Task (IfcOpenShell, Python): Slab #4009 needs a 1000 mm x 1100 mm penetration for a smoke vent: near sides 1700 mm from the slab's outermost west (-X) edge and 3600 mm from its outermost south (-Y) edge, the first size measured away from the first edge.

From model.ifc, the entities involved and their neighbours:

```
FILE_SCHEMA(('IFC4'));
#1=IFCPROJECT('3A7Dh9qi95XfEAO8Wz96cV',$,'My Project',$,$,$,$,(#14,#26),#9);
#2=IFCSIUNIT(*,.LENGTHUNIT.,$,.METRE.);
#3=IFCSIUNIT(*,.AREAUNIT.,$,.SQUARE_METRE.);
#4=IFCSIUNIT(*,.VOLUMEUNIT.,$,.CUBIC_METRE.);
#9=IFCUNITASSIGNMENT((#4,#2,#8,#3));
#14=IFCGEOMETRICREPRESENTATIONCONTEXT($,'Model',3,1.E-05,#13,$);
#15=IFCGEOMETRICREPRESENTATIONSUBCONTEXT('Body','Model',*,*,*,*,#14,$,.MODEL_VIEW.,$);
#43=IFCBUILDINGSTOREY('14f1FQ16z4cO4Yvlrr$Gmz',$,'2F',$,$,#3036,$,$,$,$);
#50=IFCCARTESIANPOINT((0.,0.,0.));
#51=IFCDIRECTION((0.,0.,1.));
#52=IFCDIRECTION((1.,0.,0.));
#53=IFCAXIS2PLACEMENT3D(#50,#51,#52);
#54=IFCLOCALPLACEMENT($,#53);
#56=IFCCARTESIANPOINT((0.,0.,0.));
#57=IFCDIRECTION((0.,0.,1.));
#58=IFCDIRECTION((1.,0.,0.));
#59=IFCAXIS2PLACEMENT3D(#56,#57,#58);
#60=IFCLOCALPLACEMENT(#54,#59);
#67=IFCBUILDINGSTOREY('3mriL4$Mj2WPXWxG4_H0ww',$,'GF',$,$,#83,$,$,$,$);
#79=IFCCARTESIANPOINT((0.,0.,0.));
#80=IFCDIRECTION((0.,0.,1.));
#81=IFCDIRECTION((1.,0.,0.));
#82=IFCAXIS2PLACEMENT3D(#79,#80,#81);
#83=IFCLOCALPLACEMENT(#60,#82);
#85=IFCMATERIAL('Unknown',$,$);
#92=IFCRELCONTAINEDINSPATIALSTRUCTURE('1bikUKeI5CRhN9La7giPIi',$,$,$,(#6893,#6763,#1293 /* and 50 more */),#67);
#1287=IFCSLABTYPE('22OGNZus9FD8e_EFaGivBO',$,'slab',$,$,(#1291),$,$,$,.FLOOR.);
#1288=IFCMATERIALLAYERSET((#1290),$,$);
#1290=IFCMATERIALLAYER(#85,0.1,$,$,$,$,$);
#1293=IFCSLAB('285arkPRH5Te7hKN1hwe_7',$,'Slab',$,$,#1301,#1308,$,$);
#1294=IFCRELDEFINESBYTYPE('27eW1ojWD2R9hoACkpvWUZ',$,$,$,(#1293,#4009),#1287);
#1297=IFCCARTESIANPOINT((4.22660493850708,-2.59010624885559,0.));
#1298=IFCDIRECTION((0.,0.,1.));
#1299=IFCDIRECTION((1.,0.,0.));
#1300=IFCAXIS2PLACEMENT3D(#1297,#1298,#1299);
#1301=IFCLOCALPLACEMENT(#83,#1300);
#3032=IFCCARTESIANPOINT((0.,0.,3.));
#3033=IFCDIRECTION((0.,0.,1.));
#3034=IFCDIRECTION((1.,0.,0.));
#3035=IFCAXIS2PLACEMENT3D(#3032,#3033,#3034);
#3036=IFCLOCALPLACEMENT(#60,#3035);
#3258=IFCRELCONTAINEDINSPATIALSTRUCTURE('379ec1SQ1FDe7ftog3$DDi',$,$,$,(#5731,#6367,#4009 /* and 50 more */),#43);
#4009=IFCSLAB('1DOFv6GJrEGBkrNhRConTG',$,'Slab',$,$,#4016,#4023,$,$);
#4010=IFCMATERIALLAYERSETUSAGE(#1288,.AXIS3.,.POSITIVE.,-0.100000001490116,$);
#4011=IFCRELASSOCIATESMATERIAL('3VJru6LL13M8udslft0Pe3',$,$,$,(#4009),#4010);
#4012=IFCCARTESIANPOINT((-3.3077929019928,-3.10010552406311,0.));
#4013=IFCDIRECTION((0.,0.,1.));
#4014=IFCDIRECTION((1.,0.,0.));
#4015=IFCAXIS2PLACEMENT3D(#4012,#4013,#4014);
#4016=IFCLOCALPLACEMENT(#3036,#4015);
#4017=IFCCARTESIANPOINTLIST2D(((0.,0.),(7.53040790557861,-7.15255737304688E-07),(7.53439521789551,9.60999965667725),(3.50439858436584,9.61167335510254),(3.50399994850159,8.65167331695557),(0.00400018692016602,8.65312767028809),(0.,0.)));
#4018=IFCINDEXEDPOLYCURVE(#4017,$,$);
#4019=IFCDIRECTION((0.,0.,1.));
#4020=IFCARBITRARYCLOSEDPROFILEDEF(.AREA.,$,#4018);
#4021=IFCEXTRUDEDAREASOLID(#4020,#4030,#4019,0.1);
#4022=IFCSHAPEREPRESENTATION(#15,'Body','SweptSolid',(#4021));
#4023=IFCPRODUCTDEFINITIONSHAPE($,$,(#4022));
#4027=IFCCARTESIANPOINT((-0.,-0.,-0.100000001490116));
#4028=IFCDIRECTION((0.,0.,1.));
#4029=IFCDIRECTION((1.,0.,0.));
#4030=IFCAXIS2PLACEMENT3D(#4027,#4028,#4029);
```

```python
import numpy as np
import ifcopenshell
import ifcopenshell.api.feature
import ifcopenshell.api.geometry
import ifcopenshell.api.root
import ifcopenshell.geom
import ifcopenshell.util.placement
import ifcopenshell.util.representation
import ifcopenshell.util.shape
import ifcopenshell.util.unit

model = ifcopenshell.open("model.ifc")
unit_scale = ifcopenshell.util.unit.calculate_unit_scale(model)
settings = ifcopenshell.geom.settings()


def volume(element):
    """Net volume in cubic metres, openings subtracted."""
    shape = ifcopenshell.geom.create_shape(settings, element)
    return ifcopenshell.util.shape.get_volume(shape.geometry)


slab = model.by_guid("1DOFv6GJrEGBkrNhRConTG")
before = volume(slab)

# Extent in the slab's own axes, in metres. The edges named are its -X and -Y sides.
slab_shape = ifcopenshell.geom.create_shape(settings, slab)
vertices = ifcopenshell.util.shape.get_vertices(slab_shape.geometry)
x_min, y_min, bottom = vertices.min(axis=0)
top = vertices[:, 2].max()

opening = ifcopenshell.api.root.create_entity(model, ifc_class="IfcOpeningElement", name="Smoke vent opening", predefined_type="OPENING")
context = ifcopenshell.util.representation.get_context(model, "Model", "Body", "MODEL_VIEW")
width, depth = 1, 1.1
outline = [(0.0, 0.0), (width, 0.0), (width, depth), (0.0, depth), (0.0, 0.0)]
# Overshoot both faces by 50 mm so the cut is clean.
shape = ifcopenshell.api.geometry.add_slab_representation(
    model, context=context, depth=top - bottom + 0.1, polyline=outline
)
ifcopenshell.api.geometry.assign_representation(model, product=opening, representation=shape)

matrix = ifcopenshell.util.placement.get_local_placement(slab.ObjectPlacement)
matrix[:, 3] = matrix @ np.append(np.array([x_min + 1.7, y_min + 3.6, bottom - 0.05]) / unit_scale, 1.0)
ifcopenshell.api.geometry.edit_object_placement(model, product=opening, matrix=matrix, is_si=False)
ifcopenshell.api.feature.add_feature(model, feature=opening, element=slab)

after = volume(slab)

print(f"slab volume {before:.3f} -> {after:.3f} m3")

model.write("model_updated.ifc")
```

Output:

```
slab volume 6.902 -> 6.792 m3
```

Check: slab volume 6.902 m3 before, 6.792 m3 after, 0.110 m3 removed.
